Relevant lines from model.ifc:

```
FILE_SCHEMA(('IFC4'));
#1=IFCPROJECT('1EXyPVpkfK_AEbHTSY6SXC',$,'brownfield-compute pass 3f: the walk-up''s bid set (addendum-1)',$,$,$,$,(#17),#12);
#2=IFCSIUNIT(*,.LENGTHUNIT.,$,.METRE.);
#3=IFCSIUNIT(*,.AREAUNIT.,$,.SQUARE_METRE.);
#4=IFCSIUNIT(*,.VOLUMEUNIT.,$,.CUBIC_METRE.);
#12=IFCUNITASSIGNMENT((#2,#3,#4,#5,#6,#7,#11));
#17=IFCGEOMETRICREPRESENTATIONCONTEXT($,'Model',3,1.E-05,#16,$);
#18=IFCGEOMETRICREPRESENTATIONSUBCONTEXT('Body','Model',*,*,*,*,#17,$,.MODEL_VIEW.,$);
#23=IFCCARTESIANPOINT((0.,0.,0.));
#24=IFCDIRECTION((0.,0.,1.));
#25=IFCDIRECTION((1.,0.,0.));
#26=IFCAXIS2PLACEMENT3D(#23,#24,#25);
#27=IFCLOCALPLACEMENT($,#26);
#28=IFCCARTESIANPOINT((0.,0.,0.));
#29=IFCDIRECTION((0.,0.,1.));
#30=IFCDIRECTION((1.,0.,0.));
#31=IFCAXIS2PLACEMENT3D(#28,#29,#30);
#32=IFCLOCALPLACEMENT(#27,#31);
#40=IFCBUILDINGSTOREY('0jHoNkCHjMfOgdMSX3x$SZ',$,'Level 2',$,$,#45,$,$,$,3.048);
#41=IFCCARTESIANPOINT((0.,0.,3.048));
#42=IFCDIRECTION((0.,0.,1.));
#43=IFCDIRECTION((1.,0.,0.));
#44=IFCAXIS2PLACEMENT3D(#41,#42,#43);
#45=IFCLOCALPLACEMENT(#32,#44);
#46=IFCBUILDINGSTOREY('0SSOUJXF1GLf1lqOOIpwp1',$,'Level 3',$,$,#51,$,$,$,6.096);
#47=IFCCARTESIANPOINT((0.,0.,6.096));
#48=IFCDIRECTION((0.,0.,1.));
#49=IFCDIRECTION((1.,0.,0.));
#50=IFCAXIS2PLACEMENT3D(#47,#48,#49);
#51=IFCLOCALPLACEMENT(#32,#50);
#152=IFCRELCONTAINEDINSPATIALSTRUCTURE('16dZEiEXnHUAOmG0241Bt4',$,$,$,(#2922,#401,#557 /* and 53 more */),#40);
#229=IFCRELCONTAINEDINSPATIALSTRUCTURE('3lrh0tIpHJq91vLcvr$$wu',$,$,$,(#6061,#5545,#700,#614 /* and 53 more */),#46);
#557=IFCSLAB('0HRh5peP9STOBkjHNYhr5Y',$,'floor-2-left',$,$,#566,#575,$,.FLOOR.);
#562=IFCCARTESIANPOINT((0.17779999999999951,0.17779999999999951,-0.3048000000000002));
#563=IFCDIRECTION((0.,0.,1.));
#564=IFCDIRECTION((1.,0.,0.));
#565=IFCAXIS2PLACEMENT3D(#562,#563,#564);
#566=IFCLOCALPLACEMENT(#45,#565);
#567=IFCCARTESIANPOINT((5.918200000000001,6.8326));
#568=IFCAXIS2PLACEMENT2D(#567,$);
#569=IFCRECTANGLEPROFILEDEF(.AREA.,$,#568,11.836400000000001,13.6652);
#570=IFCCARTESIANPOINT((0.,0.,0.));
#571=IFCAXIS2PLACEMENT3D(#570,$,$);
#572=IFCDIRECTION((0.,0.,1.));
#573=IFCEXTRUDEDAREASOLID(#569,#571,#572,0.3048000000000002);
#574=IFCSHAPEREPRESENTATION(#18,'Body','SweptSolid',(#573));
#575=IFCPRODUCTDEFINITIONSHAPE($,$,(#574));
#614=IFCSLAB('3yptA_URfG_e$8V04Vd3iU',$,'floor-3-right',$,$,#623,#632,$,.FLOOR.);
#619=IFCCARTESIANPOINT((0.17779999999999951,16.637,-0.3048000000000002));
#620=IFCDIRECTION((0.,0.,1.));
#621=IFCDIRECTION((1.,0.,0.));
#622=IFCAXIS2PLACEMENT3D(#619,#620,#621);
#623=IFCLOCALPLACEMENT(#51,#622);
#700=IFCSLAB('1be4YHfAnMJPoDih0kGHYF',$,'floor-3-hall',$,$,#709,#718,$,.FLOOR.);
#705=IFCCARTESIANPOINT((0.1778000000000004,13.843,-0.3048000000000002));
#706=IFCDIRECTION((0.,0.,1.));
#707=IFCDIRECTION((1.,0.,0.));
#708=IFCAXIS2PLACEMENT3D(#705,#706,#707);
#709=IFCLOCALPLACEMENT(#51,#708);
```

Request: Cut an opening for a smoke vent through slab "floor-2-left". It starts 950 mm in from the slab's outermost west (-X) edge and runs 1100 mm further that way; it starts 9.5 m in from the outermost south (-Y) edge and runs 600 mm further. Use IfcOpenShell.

```python
import numpy as np
import ifcopenshell
import ifcopenshell.api.feature
import ifcopenshell.api.geometry
import ifcopenshell.api.root
import ifcopenshell.geom
import ifcopenshell.util.placement
import ifcopenshell.util.representation
import ifcopenshell.util.shape
import ifcopenshell.util.unit

model = ifcopenshell.open("model.ifc")
unit_scale = ifcopenshell.util.unit.calculate_unit_scale(model)
settings = ifcopenshell.geom.settings()


def volume(element):
    """Net volume in cubic metres, openings subtracted."""
    shape = ifcopenshell.geom.create_shape(settings, element)
    return ifcopenshell.util.shape.get_volume(shape.geometry)


slab = model.by_guid("0HRh5peP9STOBkjHNYhr5Y")
before = volume(slab)

# Extent in the slab's own axes, in metres. The edges named are its -X and -Y sides.
slab_shape = ifcopenshell.geom.create_shape(settings, slab)
vertices = ifcopenshell.util.shape.get_vertices(slab_shape.geometry)
x_min, y_min, bottom = vertices.min(axis=0)
top = vertices[:, 2].max()

opening = ifcopenshell.api.root.create_entity(model, ifc_class="IfcOpeningElement", name="Smoke vent opening", predefined_type="OPENING")
context = ifcopenshell.util.representation.get_context(model, "Model", "Body", "MODEL_VIEW")
width, depth = 1.1, 0.6
outline = [(0.0, 0.0), (width, 0.0), (width, depth), (0.0, depth), (0.0, 0.0)]
# Overshoot both faces by 50 mm so the cut is clean.
shape = ifcopenshell.api.geometry.add_slab_representation(
    model, context=context, depth=top - bottom + 0.1, polyline=outline
)
ifcopenshell.api.geometry.assign_representation(model, product=opening, representation=shape)

matrix = ifcopenshell.util.placement.get_local_placement(slab.ObjectPlacement)
matrix[:, 3] = matrix @ np.append(np.array([x_min + 0.95, y_min + 9.5, bottom - 0.05]) / unit_scale, 1.0)
ifcopenshell.api.geometry.edit_object_placement(model, product=opening, matrix=matrix, is_si=False)
ifcopenshell.api.feature.add_feature(model, feature=opening, element=slab)

after = volume(slab)

print(f"slab volume {before:.3f} -> {after:.3f} m3")

model.write("model_v2.ifc")
```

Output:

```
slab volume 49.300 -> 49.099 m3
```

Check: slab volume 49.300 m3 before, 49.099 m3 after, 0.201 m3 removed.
